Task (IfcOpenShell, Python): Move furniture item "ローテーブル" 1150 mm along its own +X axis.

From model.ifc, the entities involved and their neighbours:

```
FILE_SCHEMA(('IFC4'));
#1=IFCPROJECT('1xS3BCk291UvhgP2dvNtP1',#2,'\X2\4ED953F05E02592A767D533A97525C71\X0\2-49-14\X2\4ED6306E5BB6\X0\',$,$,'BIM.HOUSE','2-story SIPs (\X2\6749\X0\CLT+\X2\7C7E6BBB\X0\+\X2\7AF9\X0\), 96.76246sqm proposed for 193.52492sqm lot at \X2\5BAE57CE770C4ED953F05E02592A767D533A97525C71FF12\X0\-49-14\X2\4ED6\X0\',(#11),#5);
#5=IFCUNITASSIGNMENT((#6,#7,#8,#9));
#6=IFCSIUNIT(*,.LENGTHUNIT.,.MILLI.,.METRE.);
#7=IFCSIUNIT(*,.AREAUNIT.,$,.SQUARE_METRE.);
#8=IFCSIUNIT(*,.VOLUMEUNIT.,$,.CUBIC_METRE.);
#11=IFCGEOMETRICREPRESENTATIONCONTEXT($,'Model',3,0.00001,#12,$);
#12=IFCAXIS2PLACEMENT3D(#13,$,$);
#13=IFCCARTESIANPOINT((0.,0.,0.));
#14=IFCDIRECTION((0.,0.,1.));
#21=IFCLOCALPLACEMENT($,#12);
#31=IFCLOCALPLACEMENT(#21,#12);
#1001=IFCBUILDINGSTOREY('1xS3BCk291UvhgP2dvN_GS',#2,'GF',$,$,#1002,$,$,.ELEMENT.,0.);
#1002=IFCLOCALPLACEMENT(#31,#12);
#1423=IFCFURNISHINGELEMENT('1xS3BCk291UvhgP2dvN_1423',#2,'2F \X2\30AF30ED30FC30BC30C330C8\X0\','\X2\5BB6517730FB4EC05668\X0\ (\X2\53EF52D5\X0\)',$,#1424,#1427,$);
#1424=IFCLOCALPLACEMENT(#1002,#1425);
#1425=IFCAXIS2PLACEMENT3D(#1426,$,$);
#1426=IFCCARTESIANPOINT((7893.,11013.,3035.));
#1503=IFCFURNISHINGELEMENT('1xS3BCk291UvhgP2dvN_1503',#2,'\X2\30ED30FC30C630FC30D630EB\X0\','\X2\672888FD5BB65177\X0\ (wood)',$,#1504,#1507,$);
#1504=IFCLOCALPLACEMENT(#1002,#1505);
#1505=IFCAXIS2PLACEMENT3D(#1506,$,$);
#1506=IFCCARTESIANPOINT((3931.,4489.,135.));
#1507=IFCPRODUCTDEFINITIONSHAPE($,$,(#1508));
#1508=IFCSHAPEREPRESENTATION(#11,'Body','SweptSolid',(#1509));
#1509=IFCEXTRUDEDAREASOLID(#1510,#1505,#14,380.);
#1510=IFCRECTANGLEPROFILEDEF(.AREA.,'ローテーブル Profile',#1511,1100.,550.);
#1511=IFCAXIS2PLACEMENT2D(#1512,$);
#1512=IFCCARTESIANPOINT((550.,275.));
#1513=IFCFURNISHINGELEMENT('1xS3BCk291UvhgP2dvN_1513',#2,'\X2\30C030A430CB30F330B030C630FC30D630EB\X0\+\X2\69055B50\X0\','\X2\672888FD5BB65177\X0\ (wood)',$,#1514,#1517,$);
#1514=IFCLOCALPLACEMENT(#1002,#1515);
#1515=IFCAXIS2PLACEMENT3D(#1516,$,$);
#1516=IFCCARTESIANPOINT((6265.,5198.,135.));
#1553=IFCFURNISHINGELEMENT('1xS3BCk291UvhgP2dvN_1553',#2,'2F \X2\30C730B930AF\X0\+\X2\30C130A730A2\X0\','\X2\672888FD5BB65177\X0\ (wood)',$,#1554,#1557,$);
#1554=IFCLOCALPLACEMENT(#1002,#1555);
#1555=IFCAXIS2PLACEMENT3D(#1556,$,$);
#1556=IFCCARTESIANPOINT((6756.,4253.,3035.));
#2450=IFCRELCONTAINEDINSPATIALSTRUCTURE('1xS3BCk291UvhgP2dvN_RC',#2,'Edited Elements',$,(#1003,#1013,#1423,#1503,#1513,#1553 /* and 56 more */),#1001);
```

```python
import ifcopenshell
import ifcopenshell.api.geometry
import ifcopenshell.util.placement
import ifcopenshell.util.unit

model = ifcopenshell.open("model.ifc")
unit_scale = ifcopenshell.util.unit.calculate_unit_scale(model)

item = model.by_guid("1xS3BCk291UvhgP2dvN_1503")
matrix = ifcopenshell.util.placement.get_local_placement(item.ObjectPlacement)
matrix[:3, 3] += matrix[:3, 0] * 1.15 / unit_scale
ifcopenshell.api.geometry.edit_object_placement(model, product=item, matrix=matrix, is_si=False)

print(ifcopenshell.util.placement.get_local_placement(item.ObjectPlacement).round(3) + 0.0)

model.write("model_edited.ifc")
```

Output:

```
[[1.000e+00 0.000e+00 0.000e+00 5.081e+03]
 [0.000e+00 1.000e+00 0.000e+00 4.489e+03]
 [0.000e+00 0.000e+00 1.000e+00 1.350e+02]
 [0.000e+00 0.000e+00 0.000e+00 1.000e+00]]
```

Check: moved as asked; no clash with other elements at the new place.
